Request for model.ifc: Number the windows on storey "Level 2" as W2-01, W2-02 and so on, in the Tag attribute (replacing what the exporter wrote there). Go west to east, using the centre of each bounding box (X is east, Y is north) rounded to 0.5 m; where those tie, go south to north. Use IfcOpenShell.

First a look at what the model holds.

```python
import ifcopenshell
import ifcopenshell.util.element
import ifcopenshell.util.placement

model = ifcopenshell.open("model.ifc")
print(model.schema)
storey = next(s for s in model.by_type("IfcBuildingStorey") if s.Name == "Level 2")
windows = [e for e in ifcopenshell.util.element.get_decomposition(storey) if e.is_a("IfcWindow")]
for e in sorted(windows, key=lambda e: e.id()):
    origin = ifcopenshell.util.placement.get_local_placement(e.ObjectPlacement)[:3, 3]
    print(e.id(), e.Tag, e.Name, origin.round(2) + 0.0, sep=" | ")
```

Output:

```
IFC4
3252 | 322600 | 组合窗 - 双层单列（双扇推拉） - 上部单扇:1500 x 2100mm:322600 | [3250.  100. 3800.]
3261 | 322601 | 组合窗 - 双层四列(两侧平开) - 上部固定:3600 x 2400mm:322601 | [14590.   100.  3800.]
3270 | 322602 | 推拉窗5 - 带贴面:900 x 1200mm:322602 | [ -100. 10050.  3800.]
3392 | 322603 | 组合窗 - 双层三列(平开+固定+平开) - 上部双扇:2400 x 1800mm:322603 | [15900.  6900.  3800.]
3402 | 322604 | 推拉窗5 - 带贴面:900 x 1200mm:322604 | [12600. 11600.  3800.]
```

```python
import ifcopenshell
import ifcopenshell.geom
import ifcopenshell.util.element
import ifcopenshell.util.shape

model = ifcopenshell.open("model.ifc")
settings = ifcopenshell.geom.settings()
settings.set("use-world-coords", True)


def centre(element):
    shape = ifcopenshell.geom.create_shape(settings, element)
    return ifcopenshell.util.shape.get_bbox_centroid(shape.geometry)


storey = next(s for s in model.by_type("IfcBuildingStorey") if s.Name == "Level 2")
windows = [e for e in ifcopenshell.util.element.get_decomposition(storey) if e.is_a("IfcWindow")]

# Insertion points can sit at a corner or the storey origin, so sort by the geometry (in metres).
centres = {e: centre(e) for e in windows}
windows.sort(key=lambda e: (round(centres[e][0] / 0.5), centres[e][1]))

for i, e in enumerate(windows, start=1):
    number = f"W2-{i:02d}"
    e.Tag = number
    print(e.id(), number)

model.write("model_v2.ifc")
```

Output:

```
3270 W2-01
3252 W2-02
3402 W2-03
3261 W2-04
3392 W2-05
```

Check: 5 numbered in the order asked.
